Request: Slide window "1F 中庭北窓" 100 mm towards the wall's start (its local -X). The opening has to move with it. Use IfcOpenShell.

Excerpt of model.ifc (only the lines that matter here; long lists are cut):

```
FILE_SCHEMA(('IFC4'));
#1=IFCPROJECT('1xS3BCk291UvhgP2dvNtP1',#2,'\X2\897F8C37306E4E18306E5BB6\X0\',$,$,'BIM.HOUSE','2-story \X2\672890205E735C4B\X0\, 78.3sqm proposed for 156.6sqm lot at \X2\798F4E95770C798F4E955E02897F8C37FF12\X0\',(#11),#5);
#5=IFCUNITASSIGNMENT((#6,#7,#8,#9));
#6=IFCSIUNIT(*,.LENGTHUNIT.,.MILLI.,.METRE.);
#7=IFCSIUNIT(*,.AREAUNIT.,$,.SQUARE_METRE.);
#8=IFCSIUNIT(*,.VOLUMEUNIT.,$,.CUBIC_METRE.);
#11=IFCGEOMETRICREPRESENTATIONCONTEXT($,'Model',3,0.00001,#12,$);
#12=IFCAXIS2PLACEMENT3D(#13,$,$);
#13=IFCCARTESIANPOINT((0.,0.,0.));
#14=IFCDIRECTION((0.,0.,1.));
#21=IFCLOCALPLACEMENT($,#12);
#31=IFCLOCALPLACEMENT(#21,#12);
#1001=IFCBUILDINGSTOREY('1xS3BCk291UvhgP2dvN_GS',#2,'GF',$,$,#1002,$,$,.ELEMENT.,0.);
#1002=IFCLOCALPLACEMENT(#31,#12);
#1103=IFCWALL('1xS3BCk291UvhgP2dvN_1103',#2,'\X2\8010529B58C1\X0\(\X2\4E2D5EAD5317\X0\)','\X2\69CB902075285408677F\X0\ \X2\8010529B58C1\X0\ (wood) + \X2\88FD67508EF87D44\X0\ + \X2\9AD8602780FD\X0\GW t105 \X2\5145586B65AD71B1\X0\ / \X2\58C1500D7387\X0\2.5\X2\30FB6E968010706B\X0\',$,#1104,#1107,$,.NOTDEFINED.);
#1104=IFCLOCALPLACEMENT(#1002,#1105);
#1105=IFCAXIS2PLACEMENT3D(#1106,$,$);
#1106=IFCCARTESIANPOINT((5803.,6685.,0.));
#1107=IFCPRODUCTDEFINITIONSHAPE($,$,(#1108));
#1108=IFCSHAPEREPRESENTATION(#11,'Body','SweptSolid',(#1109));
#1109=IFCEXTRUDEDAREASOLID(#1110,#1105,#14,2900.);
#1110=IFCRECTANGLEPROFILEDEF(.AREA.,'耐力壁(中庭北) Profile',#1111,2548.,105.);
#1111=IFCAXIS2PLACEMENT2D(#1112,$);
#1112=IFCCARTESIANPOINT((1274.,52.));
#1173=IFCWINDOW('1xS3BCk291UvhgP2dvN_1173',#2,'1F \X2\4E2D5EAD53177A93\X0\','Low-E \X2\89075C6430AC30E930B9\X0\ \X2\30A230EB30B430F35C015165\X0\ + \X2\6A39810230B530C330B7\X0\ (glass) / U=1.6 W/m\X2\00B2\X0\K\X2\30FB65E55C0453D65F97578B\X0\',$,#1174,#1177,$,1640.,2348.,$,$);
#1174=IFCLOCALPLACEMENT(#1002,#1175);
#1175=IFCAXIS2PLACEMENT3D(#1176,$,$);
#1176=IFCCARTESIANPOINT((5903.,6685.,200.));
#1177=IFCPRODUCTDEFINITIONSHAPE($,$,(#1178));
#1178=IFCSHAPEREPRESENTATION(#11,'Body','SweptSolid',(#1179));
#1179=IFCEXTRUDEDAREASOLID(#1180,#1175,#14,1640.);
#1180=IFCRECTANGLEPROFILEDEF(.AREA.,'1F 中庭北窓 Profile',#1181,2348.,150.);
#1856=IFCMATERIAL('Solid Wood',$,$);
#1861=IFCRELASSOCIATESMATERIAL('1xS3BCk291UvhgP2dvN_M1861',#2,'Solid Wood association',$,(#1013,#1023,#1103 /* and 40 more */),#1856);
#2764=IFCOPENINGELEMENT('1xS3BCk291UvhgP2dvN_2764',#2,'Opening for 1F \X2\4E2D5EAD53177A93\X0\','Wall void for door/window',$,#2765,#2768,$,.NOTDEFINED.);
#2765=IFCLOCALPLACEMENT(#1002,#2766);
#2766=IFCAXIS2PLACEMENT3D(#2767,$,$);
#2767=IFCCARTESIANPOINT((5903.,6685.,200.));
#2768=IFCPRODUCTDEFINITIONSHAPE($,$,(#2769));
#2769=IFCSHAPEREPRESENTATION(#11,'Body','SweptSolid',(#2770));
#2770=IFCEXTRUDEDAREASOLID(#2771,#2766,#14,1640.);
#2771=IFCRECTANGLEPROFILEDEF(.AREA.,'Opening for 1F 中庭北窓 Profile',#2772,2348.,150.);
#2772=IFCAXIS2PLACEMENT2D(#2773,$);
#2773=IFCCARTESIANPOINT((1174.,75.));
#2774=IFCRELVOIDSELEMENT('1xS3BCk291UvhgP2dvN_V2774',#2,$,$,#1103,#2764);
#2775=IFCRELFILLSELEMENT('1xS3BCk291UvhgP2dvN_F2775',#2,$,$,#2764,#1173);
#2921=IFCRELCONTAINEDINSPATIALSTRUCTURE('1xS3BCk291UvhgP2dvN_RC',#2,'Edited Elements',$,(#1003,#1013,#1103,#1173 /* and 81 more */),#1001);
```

```python
import ifcopenshell
import ifcopenshell.api.geometry
import ifcopenshell.util.placement
import ifcopenshell.util.unit

model = ifcopenshell.open("model.ifc")
unit_scale = ifcopenshell.util.unit.calculate_unit_scale(model)

window = model.by_id(1173)
opening = window.FillsVoids[0].RelatingOpeningElement
wall = opening.VoidsElements[0].RelatingBuildingElement

wall_matrix = ifcopenshell.util.placement.get_local_placement(wall.ObjectPlacement)
shift = wall_matrix[:3, 0] * -0.1 / unit_scale
before = ifcopenshell.util.placement.get_local_placement(window.ObjectPlacement)[:3, 3].copy()

# The window is not placed relative to its opening, so move both.
for product in (opening, window):
    matrix = ifcopenshell.util.placement.get_local_placement(product.ObjectPlacement)
    matrix[:3, 3] += shift
    ifcopenshell.api.geometry.edit_object_placement(model, product=product, matrix=matrix, is_si=False)

after = ifcopenshell.util.placement.get_local_placement(window.ObjectPlacement)[:3, 3]
print("window moved by", (after - before).round(3) + 0.0)

model.write("model_edited.ifc")
```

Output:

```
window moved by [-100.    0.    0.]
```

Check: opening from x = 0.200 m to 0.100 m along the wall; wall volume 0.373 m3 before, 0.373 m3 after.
